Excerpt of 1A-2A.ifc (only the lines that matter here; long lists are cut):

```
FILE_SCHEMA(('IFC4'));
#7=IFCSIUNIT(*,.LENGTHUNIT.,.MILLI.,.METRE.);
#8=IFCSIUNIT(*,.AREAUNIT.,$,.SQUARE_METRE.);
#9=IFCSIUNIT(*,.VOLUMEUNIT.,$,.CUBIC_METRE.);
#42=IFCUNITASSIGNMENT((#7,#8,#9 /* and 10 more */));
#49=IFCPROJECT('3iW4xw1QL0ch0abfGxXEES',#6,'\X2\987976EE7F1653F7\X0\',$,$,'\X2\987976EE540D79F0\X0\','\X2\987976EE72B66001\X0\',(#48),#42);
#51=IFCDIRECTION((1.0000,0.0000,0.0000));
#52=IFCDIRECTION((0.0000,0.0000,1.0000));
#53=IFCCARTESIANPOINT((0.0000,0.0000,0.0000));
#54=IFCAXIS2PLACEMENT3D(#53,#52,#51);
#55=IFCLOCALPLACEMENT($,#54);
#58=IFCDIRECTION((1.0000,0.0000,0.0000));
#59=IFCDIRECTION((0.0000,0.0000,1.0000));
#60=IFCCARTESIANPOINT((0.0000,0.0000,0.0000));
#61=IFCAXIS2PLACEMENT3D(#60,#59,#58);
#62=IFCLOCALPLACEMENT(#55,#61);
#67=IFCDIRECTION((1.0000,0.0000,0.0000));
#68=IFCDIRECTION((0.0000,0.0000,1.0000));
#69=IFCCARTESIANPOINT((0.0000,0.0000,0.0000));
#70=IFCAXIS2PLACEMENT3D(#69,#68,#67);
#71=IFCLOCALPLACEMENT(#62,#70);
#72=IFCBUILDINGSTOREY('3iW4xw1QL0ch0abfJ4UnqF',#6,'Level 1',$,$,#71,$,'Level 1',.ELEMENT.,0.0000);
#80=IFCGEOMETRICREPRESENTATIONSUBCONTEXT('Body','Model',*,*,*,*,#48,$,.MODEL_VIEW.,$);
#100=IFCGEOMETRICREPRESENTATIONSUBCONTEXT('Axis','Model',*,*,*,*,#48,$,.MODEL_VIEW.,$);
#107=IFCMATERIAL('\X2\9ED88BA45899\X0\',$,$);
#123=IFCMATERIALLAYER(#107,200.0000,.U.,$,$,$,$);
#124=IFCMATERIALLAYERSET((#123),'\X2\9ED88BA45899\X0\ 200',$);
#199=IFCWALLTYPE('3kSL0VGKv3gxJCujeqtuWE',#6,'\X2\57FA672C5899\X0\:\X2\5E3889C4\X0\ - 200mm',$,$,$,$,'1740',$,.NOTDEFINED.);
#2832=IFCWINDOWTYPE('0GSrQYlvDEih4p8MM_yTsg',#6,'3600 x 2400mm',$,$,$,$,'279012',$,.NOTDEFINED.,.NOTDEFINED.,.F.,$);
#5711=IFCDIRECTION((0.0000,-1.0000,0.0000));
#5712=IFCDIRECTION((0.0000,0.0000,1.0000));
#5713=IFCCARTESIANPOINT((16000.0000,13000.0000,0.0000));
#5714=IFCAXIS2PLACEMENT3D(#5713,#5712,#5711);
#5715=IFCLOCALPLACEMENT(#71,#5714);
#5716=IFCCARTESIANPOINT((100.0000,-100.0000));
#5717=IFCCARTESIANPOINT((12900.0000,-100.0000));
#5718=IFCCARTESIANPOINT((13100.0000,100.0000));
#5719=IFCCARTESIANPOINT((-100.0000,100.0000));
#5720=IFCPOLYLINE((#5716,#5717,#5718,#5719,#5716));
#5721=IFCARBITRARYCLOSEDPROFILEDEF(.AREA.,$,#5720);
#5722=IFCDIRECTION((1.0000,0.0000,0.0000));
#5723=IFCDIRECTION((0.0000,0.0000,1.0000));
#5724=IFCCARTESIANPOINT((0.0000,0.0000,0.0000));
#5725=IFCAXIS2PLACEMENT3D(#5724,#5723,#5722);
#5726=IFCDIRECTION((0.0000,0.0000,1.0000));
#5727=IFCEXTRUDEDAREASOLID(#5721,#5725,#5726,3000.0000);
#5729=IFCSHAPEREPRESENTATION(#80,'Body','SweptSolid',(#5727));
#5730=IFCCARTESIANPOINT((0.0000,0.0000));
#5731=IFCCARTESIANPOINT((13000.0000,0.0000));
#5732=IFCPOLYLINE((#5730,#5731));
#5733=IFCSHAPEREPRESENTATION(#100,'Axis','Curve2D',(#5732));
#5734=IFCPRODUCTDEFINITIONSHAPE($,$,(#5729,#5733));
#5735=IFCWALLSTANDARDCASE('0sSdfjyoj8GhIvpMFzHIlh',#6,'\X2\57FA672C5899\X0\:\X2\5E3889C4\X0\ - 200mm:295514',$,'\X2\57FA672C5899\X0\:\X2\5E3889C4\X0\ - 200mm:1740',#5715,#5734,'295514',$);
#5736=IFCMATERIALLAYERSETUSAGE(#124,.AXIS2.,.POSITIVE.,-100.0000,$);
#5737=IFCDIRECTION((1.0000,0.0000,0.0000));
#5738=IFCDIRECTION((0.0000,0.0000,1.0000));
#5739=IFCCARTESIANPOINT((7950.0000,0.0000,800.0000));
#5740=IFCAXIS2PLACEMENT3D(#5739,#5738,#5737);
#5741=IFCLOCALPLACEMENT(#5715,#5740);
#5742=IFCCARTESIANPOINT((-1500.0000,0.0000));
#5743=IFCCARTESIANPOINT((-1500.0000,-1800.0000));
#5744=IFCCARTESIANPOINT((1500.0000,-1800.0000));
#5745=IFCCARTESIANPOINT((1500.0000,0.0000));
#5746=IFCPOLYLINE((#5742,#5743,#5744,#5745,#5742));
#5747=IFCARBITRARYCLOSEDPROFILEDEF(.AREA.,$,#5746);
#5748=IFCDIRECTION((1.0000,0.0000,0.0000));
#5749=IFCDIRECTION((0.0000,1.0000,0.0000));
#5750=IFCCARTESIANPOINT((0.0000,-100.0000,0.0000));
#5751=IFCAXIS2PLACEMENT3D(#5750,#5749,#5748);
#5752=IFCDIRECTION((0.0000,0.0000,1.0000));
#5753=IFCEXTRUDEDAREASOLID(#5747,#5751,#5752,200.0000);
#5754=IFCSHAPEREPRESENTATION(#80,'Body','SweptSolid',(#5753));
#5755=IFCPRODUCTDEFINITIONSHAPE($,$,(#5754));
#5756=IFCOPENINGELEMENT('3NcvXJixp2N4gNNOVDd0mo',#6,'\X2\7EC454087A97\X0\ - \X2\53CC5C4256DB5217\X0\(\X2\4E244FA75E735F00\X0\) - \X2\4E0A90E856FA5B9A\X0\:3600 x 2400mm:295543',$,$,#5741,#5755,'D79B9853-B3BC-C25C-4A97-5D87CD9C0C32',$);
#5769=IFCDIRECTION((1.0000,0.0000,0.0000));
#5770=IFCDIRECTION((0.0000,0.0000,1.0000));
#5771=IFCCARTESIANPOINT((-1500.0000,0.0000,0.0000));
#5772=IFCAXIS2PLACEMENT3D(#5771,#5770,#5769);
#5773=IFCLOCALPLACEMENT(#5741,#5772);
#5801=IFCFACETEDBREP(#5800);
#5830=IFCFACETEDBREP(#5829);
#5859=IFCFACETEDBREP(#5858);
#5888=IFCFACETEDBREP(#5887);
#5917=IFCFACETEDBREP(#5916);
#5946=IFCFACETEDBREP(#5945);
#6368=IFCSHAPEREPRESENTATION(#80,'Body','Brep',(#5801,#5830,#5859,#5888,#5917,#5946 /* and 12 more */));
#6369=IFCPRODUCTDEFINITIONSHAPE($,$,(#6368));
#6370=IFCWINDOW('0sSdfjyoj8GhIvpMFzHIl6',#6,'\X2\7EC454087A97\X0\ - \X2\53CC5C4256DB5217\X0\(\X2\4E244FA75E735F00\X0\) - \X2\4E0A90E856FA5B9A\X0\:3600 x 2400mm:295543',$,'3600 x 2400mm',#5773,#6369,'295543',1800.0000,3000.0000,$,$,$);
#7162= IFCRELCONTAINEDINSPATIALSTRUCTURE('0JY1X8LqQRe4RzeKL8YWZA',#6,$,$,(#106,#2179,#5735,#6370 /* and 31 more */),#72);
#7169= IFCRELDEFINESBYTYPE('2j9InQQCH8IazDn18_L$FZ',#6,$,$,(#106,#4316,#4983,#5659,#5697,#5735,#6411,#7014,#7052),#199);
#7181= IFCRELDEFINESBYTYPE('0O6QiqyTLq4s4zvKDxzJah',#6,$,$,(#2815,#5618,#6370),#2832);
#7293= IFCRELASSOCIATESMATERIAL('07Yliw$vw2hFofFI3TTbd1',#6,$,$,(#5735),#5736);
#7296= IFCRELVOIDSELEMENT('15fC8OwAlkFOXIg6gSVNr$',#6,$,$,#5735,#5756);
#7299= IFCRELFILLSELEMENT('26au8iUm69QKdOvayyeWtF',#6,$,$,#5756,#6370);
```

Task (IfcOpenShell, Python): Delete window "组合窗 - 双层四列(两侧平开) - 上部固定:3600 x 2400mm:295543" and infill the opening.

```python
import ifcopenshell
import ifcopenshell.api.feature
import ifcopenshell.api.root
import ifcopenshell.geom
import ifcopenshell.util.shape

model = ifcopenshell.open("1A-2A.ifc")
settings = ifcopenshell.geom.settings()


def volume(element):
    """Net volume in cubic metres, openings subtracted."""
    shape = ifcopenshell.geom.create_shape(settings, element)
    return ifcopenshell.util.shape.get_volume(shape.geometry)


window = model.by_guid("0sSdfjyoj8GhIvpMFzHIl6")
opening = window.FillsVoids[0].RelatingOpeningElement
wall = opening.VoidsElements[0].RelatingBuildingElement
before = volume(wall)

ifcopenshell.api.root.remove_product(model, product=window)
ifcopenshell.api.feature.remove_feature(model, feature=opening)

after = volume(wall)

print(f"wall volume {before:.3f} -> {after:.3f} m3")

model.write("1A-2A_updated.ifc")
```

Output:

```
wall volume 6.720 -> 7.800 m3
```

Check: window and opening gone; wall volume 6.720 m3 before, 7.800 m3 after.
